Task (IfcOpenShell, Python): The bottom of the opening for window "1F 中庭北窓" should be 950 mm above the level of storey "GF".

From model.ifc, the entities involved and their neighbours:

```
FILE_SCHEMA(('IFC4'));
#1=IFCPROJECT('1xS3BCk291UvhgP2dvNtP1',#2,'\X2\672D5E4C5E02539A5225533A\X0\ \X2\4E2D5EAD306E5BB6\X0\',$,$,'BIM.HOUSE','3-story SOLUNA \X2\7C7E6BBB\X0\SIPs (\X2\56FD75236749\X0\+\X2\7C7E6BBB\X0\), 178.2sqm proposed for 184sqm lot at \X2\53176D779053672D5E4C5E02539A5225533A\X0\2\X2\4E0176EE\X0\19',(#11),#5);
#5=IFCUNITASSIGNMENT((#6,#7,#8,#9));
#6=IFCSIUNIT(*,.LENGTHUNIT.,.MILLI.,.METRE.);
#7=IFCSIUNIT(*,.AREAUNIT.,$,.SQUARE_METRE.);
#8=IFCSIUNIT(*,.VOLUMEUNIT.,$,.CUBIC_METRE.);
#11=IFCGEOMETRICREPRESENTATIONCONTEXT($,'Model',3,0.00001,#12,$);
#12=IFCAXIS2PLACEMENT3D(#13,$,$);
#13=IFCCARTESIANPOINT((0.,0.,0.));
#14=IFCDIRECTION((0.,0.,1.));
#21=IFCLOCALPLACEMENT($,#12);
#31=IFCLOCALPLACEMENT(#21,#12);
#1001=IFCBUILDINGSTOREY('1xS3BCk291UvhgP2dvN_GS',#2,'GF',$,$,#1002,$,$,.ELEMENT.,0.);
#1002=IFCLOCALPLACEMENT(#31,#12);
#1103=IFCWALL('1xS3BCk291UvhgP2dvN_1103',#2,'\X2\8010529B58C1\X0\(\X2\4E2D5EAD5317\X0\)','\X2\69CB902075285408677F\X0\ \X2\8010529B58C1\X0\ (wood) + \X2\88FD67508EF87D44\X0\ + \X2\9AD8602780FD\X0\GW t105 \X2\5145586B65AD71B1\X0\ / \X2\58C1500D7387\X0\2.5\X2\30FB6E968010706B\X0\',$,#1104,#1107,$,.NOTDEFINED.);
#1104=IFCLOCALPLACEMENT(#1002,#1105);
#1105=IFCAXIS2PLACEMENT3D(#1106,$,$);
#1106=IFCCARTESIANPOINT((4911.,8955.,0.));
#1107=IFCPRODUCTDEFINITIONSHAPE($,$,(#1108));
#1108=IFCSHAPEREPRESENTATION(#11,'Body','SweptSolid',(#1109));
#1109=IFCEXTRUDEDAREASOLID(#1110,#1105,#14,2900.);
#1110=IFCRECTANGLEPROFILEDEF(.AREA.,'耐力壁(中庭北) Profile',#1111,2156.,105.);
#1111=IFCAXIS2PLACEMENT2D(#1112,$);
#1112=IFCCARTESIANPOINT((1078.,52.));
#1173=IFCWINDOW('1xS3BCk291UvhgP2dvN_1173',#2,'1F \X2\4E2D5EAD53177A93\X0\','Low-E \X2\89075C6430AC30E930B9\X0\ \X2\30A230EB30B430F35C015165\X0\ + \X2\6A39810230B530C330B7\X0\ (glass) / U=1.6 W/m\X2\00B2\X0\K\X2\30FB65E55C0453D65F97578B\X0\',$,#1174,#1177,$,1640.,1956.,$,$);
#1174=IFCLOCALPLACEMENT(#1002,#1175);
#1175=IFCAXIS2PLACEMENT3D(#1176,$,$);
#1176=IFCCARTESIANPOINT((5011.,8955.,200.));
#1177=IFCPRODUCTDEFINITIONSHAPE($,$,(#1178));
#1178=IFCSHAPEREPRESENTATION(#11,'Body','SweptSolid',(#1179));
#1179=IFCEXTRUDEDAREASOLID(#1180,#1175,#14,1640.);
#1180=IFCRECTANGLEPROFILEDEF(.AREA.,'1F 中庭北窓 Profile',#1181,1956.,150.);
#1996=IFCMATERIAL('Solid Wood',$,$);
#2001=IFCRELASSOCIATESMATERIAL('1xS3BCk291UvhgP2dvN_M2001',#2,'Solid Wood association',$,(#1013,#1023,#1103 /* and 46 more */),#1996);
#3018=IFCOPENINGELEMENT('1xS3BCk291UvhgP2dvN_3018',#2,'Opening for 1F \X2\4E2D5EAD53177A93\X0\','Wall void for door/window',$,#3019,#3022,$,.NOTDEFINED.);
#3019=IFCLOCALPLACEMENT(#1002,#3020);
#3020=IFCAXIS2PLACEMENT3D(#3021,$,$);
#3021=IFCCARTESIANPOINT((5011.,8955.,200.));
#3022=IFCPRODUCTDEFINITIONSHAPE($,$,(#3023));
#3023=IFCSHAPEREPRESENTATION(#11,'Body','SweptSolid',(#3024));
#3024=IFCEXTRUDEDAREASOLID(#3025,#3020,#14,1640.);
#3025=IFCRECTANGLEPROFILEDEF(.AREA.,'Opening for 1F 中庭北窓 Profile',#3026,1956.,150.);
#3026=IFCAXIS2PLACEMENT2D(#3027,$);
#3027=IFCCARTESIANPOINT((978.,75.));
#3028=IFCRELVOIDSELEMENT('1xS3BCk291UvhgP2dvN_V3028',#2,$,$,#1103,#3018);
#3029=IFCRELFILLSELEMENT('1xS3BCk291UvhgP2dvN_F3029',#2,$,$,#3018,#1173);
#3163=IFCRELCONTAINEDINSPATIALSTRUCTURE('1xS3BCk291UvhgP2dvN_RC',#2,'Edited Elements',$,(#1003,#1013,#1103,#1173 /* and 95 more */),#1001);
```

```python
import numpy as np
import ifcopenshell
import ifcopenshell.api.geometry
import ifcopenshell.geom
import ifcopenshell.util.element
import ifcopenshell.util.placement
import ifcopenshell.util.shape
import ifcopenshell.util.unit

model = ifcopenshell.open("model.ifc")
unit_scale = ifcopenshell.util.unit.calculate_unit_scale(model)

window = model.by_id(1173)
opening = window.FillsVoids[0].RelatingOpeningElement
storey = ifcopenshell.util.element.get_container(window, ifc_class="IfcBuildingStorey")
level = ifcopenshell.util.placement.get_local_placement(storey.ObjectPlacement)[2, 3]

# The opening's origin need not be at the sill, so measure its lowest point.
shape = ifcopenshell.geom.create_shape(ifcopenshell.geom.settings(), opening)
bottom = ifcopenshell.util.shape.get_shape_bottom_elevation(shape, shape.geometry) / unit_scale
dz = level + 0.95 / unit_scale - bottom

shift = np.array([0.0, 0.0, dz])
# The window is not placed relative to its opening, so move both.
for product in (opening, window):
    matrix = ifcopenshell.util.placement.get_local_placement(product.ObjectPlacement)
    matrix[:3, 3] += shift
    ifcopenshell.api.geometry.edit_object_placement(model, product=product, matrix=matrix, is_si=False)

print(f"moved by {dz * unit_scale:+.3f} m")

model.write("model-out.ifc")
```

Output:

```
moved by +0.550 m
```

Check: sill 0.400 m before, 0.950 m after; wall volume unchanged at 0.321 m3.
